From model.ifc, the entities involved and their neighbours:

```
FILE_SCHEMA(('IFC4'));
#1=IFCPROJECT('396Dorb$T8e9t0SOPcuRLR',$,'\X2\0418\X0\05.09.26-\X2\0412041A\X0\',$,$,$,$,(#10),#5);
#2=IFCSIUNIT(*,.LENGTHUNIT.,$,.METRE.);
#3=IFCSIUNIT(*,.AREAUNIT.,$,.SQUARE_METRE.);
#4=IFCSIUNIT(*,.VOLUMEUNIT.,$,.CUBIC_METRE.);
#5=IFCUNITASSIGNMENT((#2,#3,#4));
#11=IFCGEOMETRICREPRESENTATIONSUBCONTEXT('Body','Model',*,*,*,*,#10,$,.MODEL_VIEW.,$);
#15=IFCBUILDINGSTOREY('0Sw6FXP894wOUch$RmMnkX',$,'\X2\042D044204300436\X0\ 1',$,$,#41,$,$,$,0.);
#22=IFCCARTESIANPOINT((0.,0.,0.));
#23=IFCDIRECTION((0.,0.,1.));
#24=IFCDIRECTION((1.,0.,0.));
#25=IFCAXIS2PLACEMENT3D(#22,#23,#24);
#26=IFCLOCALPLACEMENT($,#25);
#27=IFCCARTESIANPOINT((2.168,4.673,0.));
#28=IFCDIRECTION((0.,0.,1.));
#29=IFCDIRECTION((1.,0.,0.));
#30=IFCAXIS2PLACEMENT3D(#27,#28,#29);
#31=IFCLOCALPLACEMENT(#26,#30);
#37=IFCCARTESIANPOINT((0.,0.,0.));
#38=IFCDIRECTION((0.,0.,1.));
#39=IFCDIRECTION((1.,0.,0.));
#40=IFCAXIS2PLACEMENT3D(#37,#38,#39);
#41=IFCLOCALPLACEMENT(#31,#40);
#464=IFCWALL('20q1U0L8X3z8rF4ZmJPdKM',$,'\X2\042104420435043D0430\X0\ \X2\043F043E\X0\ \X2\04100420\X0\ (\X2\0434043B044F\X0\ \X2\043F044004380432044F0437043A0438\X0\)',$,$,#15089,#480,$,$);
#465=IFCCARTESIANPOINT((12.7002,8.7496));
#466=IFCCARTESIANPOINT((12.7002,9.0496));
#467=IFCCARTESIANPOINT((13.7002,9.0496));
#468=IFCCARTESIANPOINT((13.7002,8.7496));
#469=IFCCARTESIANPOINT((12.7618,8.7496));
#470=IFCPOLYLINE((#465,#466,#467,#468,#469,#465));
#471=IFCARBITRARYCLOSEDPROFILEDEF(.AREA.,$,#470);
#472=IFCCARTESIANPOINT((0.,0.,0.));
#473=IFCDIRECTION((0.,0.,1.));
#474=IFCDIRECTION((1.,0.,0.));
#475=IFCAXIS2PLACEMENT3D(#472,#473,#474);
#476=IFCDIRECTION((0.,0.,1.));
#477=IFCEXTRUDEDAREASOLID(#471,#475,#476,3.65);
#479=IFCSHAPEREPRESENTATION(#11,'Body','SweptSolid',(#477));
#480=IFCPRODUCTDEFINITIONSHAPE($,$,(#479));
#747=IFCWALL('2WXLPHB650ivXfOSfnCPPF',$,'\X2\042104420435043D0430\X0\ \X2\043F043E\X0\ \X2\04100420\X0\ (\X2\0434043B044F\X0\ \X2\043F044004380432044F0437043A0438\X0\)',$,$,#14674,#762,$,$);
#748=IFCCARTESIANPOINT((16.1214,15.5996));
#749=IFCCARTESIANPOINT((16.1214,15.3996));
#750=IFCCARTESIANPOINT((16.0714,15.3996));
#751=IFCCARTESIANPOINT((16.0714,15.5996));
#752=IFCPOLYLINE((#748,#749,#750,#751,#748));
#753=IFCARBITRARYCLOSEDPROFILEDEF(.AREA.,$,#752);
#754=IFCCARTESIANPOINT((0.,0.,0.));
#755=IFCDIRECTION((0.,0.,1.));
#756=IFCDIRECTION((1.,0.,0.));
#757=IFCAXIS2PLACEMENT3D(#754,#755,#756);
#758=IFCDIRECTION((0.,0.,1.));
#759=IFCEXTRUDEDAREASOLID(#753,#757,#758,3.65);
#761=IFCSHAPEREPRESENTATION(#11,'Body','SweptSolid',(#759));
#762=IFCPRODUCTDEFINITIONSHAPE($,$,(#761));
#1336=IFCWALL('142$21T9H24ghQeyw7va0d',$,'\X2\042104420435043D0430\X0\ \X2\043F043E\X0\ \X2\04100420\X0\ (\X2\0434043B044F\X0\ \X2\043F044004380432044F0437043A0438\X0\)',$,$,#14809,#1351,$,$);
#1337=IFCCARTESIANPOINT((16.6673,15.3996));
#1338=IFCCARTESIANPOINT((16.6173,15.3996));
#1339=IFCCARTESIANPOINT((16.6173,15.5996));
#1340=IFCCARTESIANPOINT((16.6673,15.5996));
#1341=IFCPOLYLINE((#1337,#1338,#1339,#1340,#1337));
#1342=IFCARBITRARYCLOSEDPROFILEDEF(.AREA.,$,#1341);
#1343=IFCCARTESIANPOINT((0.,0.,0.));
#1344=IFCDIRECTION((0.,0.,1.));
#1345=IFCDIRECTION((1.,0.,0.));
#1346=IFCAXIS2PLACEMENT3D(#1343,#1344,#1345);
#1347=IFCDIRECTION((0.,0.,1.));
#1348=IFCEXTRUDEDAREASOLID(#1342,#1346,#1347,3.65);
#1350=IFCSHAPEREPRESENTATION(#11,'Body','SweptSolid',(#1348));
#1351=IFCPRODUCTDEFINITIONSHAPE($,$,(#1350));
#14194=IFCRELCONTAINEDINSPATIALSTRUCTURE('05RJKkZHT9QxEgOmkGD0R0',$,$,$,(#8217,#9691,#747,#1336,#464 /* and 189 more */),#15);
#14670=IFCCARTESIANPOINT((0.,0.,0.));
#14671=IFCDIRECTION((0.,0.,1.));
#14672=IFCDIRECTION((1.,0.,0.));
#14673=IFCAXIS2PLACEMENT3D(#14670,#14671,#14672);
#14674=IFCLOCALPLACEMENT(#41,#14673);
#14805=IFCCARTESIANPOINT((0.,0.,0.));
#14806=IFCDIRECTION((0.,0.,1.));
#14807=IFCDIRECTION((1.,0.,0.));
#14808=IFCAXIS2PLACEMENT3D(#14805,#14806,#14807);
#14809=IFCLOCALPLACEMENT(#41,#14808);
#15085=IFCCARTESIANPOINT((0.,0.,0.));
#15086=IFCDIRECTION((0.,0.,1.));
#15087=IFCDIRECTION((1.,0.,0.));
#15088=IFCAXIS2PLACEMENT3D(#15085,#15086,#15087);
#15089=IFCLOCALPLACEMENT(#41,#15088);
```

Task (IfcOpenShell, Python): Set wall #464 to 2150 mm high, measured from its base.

```python
import ifcopenshell
import ifcopenshell.geom
import ifcopenshell.util.representation
import ifcopenshell.util.shape

model = ifcopenshell.open("model.ifc")
settings = ifcopenshell.geom.settings()


def volume(element):
    """Net volume in cubic metres, openings subtracted."""
    shape = ifcopenshell.geom.create_shape(settings, element)
    return ifcopenshell.util.shape.get_volume(shape.geometry)


wall = model.by_guid("20q1U0L8X3z8rF4ZmJPdKM")
before = volume(wall)

body = ifcopenshell.util.representation.get_representation(wall, "Model", "Body")
solid = body.Items[0]
old_height = solid.Depth
solid.Depth = 2.15
after = volume(wall)

print(f"height {old_height:g} -> {solid.Depth:g}, volume {before:.3f} -> {after:.3f} m3")

model.write("model_rev.ifc")
```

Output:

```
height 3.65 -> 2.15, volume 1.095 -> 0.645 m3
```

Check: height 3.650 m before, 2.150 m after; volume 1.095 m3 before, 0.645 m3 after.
